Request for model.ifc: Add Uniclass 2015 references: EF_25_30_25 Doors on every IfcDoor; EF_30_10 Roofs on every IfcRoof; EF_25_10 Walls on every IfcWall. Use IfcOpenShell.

First a look at what the model holds.

```python
import ifcopenshell

model = ifcopenshell.open("model.ifc")
print(model.schema)
print("classifications:", [c.Name for c in model.by_type("IfcClassification")])
for ifc_class in ("IfcDoor", "IfcRoof", "IfcStair", "IfcWall", "IfcWindow"):
    print(ifc_class, len(model.by_type(ifc_class)))
```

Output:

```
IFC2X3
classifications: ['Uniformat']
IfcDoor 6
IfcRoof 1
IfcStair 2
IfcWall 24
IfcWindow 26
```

```python
import ifcopenshell
import ifcopenshell.api.classification

model = ifcopenshell.open("model.ifc")

# IFC2X3 requires Source and Edition and has no link from the project to the system.
system = model.create_entity("IfcClassification", Source="NBS", Edition="2015", Name="Uniclass 2015")

codes = {
    "IfcDoor": ("EF_25_30_25", "Doors"),
    "IfcRoof": ("EF_30_10", "Roofs"),
    "IfcWall": ("EF_25_10", "Walls"),
}
for ifc_class, (code, name) in codes.items():
    products = model.by_type(ifc_class)
    ifcopenshell.api.classification.add_reference(
        model, products=products, classification=system, identification=code, name=name
    )
    print(code, len(products))

model.write("model_updated.ifc")
```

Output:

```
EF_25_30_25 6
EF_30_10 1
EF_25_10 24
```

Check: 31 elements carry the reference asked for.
